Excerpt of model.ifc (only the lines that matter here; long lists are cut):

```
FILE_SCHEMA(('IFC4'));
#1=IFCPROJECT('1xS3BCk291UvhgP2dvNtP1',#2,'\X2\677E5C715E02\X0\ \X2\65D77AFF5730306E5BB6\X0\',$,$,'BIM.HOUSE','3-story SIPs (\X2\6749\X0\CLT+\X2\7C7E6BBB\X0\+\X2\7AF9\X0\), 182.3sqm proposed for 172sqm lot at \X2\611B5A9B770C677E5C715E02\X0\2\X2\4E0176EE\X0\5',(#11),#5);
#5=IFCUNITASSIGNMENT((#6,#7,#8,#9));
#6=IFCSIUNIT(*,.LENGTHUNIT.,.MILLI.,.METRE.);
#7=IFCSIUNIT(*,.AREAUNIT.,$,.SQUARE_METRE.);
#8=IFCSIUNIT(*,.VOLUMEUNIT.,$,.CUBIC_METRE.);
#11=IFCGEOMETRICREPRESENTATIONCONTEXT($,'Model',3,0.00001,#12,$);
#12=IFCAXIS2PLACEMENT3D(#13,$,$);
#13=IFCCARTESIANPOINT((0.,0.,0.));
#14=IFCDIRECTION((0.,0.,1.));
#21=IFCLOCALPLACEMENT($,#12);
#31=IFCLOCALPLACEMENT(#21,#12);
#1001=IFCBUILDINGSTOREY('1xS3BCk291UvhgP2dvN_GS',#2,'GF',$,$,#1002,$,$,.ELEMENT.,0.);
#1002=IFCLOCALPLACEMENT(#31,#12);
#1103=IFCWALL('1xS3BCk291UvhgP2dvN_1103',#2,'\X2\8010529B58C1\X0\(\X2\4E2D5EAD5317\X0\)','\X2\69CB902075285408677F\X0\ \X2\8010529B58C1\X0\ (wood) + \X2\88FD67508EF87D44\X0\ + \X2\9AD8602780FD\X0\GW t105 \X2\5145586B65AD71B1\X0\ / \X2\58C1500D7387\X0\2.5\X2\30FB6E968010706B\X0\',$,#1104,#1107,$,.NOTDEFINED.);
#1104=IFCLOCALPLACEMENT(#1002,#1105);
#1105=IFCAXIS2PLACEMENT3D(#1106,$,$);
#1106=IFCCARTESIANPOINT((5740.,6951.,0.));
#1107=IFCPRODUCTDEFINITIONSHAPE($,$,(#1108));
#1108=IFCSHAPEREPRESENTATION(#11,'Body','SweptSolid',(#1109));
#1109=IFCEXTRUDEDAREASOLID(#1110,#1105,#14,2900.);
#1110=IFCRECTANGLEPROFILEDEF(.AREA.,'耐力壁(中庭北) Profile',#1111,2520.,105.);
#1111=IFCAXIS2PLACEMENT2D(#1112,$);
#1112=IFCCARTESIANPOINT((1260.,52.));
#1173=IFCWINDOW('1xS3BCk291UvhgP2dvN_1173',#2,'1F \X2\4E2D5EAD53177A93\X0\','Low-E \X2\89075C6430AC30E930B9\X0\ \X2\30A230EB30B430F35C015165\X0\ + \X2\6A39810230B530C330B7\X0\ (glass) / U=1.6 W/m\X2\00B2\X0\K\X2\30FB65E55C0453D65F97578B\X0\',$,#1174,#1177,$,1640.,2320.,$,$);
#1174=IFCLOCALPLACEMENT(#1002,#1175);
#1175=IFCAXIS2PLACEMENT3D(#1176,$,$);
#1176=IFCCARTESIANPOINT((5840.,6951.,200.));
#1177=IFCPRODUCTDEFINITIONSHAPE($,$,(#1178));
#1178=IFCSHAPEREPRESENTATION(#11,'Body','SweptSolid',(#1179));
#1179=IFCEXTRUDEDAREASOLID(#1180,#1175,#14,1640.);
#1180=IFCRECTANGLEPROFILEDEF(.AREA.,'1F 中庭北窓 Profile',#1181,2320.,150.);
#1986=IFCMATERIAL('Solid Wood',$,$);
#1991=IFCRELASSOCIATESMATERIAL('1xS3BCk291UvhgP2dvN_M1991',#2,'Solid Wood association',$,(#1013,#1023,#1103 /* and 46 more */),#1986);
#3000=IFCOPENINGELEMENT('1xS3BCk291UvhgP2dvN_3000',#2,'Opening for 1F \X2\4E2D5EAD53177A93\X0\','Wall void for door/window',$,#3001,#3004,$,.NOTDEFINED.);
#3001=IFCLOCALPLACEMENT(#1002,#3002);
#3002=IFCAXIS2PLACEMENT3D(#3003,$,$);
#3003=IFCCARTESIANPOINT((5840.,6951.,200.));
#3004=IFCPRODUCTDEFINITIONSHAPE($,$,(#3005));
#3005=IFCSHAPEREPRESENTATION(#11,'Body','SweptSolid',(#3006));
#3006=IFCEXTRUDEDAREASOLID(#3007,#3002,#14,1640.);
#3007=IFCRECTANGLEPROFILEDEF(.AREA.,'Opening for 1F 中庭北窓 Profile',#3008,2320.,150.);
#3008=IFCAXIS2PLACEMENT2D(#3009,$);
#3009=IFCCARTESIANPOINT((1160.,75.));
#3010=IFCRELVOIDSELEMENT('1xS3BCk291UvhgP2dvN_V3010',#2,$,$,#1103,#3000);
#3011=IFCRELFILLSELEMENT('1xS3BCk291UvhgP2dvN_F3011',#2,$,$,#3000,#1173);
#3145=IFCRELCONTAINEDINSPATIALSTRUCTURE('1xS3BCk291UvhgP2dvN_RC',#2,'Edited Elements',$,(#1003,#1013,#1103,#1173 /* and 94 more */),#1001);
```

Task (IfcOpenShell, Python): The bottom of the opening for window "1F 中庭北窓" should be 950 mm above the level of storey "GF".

```python
import numpy as np
import ifcopenshell
import ifcopenshell.api.geometry
import ifcopenshell.geom
import ifcopenshell.util.element
import ifcopenshell.util.placement
import ifcopenshell.util.shape
import ifcopenshell.util.unit

model = ifcopenshell.open("model.ifc")
unit_scale = ifcopenshell.util.unit.calculate_unit_scale(model)

window = model.by_guid("1xS3BCk291UvhgP2dvN_1173")
opening = window.FillsVoids[0].RelatingOpeningElement
storey = ifcopenshell.util.element.get_container(window, ifc_class="IfcBuildingStorey")
level = ifcopenshell.util.placement.get_local_placement(storey.ObjectPlacement)[2, 3]

# The opening's origin need not be at the sill, so measure its lowest point.
shape = ifcopenshell.geom.create_shape(ifcopenshell.geom.settings(), opening)
bottom = ifcopenshell.util.shape.get_shape_bottom_elevation(shape, shape.geometry) / unit_scale
dz = level + 0.95 / unit_scale - bottom

shift = np.array([0.0, 0.0, dz])
# The window is not placed relative to its opening, so move both.
for product in (opening, window):
    matrix = ifcopenshell.util.placement.get_local_placement(product.ObjectPlacement)
    matrix[:3, 3] += shift
    ifcopenshell.api.geometry.edit_object_placement(model, product=product, matrix=matrix, is_si=False)

print(f"moved by {dz * unit_scale:+.3f} m")

model.write("model_v2.ifc")
```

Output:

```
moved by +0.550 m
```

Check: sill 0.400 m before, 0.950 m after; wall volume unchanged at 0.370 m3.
